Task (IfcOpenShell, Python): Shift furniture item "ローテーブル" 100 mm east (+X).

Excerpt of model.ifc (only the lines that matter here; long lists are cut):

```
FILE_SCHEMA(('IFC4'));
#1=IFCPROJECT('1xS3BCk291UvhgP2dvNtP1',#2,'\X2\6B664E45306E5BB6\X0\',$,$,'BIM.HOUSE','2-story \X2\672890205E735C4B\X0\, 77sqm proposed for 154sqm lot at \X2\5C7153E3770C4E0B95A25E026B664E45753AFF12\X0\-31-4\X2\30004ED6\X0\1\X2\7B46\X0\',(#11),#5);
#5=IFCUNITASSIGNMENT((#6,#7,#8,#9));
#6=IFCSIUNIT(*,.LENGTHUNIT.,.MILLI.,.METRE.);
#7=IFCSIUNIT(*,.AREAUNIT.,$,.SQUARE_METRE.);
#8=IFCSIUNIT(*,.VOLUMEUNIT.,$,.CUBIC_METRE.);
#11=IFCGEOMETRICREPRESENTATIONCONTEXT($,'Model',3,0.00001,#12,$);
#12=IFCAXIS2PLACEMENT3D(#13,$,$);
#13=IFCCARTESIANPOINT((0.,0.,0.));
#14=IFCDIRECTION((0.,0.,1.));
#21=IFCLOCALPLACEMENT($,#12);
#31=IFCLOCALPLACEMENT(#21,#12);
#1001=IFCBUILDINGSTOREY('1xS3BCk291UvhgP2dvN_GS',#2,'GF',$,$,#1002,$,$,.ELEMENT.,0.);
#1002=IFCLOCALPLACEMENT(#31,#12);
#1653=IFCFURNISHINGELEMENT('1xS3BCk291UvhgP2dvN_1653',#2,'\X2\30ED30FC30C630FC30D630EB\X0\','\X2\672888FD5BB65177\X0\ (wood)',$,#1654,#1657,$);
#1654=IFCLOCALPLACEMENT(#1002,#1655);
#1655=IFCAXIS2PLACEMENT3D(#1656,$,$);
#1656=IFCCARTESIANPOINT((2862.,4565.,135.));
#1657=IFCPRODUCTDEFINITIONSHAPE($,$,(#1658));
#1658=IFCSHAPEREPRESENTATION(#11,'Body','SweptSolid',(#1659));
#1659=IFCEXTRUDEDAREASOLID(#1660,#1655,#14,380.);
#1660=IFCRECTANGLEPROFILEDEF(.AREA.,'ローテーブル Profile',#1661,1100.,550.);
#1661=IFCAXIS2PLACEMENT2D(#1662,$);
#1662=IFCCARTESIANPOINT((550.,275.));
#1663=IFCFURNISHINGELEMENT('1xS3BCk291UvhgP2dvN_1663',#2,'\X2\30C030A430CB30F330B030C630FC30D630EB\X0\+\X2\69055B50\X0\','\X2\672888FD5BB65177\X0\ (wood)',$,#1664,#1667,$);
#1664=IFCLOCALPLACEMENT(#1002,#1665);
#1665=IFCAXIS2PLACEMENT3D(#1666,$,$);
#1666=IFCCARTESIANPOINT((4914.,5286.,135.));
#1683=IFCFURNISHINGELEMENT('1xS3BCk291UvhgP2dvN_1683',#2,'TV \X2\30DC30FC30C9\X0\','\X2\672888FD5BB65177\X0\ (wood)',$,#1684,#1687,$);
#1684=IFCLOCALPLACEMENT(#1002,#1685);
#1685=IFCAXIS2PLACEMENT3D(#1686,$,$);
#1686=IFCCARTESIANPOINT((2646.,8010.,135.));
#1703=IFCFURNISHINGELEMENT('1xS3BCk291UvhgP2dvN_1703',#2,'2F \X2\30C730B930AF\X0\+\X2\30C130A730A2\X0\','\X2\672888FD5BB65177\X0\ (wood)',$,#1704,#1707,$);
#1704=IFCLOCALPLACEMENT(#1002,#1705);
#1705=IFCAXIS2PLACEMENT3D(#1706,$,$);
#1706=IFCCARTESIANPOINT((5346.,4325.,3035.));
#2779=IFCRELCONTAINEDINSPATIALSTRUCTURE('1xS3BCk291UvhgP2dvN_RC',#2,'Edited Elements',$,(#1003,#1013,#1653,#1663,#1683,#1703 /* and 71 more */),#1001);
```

```python
import ifcopenshell
import ifcopenshell.api.geometry
import ifcopenshell.util.placement
import ifcopenshell.util.unit

model = ifcopenshell.open("model.ifc")
unit_scale = ifcopenshell.util.unit.calculate_unit_scale(model)

item = model.by_guid("1xS3BCk291UvhgP2dvN_1653")
matrix = ifcopenshell.util.placement.get_local_placement(item.ObjectPlacement)
matrix[0, 3] += 0.1 / unit_scale
ifcopenshell.api.geometry.edit_object_placement(model, product=item, matrix=matrix, is_si=False)

print(ifcopenshell.util.placement.get_local_placement(item.ObjectPlacement).round(3) + 0.0)

model.write("model_updated.ifc")
```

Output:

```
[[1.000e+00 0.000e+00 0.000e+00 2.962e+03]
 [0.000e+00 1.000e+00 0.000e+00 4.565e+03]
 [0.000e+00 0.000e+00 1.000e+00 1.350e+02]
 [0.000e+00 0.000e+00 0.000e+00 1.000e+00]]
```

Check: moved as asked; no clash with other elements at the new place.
